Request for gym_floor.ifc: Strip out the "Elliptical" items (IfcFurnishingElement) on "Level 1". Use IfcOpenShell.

First a look at what the model holds.

```python
import ifcopenshell
import ifcopenshell.util.element

model = ifcopenshell.open("gym_floor.ifc")
print(model.schema)
storey = next(s for s in model.by_type("IfcBuildingStorey") if s.Name == "Level 1")
furniture = [e for e in ifcopenshell.util.element.get_decomposition(storey) if e.is_a("IfcFurnishingElement")]
seen = {}
for e in furniture:
    element_type = ifcopenshell.util.element.get_type(e)
    name = element_type.Name if element_type not in (None, e) else None
    seen[name] = seen.get(name, 0) + 1
for name, count in sorted(seen.items(), key=str):
    print(count, "x", name)
```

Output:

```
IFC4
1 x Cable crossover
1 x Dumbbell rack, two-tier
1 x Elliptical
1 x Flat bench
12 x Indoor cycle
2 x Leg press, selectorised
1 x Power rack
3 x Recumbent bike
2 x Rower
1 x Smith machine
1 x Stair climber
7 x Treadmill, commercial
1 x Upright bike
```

```python
import ifcopenshell
import ifcopenshell.api.root
import ifcopenshell.util.element

model = ifcopenshell.open("gym_floor.ifc")

storey = next(s for s in model.by_type("IfcBuildingStorey") if s.Name == "Level 1")
furniture = [e for e in ifcopenshell.util.element.get_decomposition(storey) if e.is_a("IfcFurnishingElement")]
targets = [e for e in furniture if (t := ifcopenshell.util.element.get_type(e)) not in (None, e) and t.Name == "Elliptical"]

for e in targets:
    ifcopenshell.api.root.remove_product(model, product=e)
print(len(targets), "removed")

model.write("gym_floor_edited.ifc")
```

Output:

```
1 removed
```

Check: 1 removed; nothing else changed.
